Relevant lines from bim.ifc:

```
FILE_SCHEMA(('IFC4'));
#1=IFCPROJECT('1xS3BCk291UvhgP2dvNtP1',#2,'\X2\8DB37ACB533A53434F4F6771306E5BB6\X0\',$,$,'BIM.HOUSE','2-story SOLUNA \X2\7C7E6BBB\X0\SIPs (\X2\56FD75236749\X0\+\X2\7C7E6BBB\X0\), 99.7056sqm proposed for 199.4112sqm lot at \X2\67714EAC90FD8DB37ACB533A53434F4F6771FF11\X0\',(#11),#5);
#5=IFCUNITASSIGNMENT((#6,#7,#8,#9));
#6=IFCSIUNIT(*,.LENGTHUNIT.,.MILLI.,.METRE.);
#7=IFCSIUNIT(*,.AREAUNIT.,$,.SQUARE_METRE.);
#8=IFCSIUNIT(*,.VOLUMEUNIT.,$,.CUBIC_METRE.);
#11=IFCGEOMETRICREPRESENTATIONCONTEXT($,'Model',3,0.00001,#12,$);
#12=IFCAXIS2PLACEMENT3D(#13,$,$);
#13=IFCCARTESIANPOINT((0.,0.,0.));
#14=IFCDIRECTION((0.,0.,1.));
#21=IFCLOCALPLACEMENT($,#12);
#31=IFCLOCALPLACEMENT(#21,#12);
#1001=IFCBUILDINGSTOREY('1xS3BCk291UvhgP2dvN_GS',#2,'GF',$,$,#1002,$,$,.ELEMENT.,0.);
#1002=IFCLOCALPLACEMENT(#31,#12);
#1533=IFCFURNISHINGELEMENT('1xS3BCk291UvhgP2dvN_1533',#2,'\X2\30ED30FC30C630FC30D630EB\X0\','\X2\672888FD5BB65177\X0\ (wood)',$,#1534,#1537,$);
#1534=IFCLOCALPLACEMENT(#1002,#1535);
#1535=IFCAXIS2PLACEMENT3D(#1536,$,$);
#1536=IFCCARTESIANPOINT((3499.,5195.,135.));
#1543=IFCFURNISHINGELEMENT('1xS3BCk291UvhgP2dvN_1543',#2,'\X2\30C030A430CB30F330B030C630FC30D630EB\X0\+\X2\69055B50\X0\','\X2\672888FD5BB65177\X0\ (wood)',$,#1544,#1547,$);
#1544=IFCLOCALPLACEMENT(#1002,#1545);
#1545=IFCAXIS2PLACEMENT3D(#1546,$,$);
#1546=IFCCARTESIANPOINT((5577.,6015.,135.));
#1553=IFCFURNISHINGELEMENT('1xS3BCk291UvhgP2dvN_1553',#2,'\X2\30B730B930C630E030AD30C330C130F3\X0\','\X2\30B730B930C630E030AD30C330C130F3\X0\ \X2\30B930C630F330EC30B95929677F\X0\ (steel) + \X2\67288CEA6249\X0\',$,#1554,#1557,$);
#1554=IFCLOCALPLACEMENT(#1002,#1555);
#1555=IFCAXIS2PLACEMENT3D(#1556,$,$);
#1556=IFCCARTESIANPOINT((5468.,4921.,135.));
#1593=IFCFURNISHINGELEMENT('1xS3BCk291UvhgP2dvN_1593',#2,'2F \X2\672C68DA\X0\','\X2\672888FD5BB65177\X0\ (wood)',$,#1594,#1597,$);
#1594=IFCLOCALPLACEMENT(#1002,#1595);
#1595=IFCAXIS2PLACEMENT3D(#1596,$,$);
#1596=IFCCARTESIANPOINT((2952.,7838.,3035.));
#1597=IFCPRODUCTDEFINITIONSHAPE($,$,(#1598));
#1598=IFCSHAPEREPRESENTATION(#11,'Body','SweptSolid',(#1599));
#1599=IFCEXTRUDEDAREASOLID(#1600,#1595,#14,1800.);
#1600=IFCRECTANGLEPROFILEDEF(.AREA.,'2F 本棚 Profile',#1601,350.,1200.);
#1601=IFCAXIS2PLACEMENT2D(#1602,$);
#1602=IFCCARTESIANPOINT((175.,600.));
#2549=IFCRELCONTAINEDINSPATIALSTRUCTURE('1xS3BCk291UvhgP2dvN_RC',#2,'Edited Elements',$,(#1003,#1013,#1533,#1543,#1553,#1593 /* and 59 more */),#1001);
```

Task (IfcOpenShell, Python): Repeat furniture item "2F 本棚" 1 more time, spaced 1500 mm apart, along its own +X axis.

```python
import ifcopenshell
import ifcopenshell.api.geometry
import ifcopenshell.api.root
import ifcopenshell.util.element
import ifcopenshell.util.placement
import ifcopenshell.util.unit

model = ifcopenshell.open("bim.ifc")
unit_scale = ifcopenshell.util.unit.calculate_unit_scale(model)


def reuse_history(source, copy):
    """copy_class also copies each property set's owner history, people and application; keep the originals."""
    for rel in copy.IsDefinedBy:
        if rel.is_a("IfcRelDefinesByProperties") and (history := rel.RelatingPropertyDefinition.OwnerHistory):
            rel.RelatingPropertyDefinition.OwnerHistory = source.OwnerHistory
            ifcopenshell.util.element.remove_deep2(model, history)


source = model.by_guid("1xS3BCk291UvhgP2dvN_1593")
base = ifcopenshell.util.placement.get_local_placement(source.ObjectPlacement)
step = base[:3, 0] * 1.5 / unit_scale

for i in range(1, 2):
    copy = ifcopenshell.api.root.copy_class(model, product=source)
    copy.Representation = ifcopenshell.util.element.copy_deep(
        model, source.Representation, exclude=["IfcGeometricRepresentationContext", "IfcRepresentationMap"]
    )
    reuse_history(source, copy)
    matrix = base.copy()
    matrix[:3, 3] += i * step
    print("added at", matrix[:3, 3].round(3) + 0.0)
    ifcopenshell.api.geometry.edit_object_placement(model, product=copy, matrix=matrix, is_si=False)

model.write("bim_updated.ifc")
```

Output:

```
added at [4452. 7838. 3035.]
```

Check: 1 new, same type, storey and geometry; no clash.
